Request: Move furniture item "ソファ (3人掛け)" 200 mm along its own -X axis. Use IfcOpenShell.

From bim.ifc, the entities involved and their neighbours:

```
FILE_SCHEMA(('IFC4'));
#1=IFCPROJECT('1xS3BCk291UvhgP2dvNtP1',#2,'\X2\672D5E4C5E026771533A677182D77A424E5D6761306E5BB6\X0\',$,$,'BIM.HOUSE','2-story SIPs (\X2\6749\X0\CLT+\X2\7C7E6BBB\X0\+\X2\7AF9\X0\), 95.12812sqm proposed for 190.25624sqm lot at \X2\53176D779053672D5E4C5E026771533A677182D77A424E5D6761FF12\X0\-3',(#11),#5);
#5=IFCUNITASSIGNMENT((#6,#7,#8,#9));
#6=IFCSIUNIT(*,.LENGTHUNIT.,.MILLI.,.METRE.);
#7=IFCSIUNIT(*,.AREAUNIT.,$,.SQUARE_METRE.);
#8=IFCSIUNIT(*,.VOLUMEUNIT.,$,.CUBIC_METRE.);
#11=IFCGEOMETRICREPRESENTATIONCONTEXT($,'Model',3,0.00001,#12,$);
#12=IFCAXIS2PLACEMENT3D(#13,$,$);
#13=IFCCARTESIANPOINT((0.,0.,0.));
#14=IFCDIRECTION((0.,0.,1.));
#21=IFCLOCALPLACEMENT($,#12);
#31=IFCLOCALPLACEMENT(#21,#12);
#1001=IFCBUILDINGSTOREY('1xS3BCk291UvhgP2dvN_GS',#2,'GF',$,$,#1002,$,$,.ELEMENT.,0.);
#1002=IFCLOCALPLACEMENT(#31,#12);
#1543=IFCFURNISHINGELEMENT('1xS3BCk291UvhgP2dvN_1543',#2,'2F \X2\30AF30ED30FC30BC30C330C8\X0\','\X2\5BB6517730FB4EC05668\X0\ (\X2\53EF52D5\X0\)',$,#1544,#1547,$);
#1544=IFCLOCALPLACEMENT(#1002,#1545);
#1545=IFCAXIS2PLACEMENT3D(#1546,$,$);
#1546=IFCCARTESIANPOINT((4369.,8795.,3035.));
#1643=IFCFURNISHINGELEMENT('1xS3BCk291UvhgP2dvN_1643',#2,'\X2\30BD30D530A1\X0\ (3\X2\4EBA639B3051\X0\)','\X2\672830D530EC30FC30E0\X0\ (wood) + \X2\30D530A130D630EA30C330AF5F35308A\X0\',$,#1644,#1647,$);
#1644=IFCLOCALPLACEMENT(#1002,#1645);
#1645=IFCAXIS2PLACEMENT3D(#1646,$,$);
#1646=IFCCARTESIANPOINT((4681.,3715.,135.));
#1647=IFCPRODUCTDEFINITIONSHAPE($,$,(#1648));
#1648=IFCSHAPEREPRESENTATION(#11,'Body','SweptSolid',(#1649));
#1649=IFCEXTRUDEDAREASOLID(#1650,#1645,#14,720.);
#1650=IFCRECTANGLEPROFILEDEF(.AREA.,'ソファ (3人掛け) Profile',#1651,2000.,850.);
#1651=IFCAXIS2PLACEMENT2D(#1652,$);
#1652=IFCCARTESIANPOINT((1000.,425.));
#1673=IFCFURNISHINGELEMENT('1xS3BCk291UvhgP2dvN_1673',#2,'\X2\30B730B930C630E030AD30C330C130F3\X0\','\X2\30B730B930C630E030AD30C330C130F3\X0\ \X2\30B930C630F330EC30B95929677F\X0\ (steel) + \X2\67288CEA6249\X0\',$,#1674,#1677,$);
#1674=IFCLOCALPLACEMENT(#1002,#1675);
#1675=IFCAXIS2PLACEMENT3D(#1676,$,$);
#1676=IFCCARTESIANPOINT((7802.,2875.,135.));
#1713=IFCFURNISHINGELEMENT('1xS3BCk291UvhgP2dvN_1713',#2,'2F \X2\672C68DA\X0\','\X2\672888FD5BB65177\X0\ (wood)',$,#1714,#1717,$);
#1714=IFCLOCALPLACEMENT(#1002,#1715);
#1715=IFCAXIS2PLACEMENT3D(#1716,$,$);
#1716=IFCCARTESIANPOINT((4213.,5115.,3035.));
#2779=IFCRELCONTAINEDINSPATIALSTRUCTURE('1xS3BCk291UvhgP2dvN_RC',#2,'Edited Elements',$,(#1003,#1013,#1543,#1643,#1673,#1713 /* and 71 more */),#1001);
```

```python
import ifcopenshell
import ifcopenshell.api.geometry
import ifcopenshell.util.placement
import ifcopenshell.util.unit

model = ifcopenshell.open("bim.ifc")
unit_scale = ifcopenshell.util.unit.calculate_unit_scale(model)

item = model.by_guid("1xS3BCk291UvhgP2dvN_1643")
matrix = ifcopenshell.util.placement.get_local_placement(item.ObjectPlacement)
matrix[:3, 3] -= matrix[:3, 0] * 0.2 / unit_scale
ifcopenshell.api.geometry.edit_object_placement(model, product=item, matrix=matrix, is_si=False)

print(ifcopenshell.util.placement.get_local_placement(item.ObjectPlacement).round(3) + 0.0)

model.write("bim_updated.ifc")
```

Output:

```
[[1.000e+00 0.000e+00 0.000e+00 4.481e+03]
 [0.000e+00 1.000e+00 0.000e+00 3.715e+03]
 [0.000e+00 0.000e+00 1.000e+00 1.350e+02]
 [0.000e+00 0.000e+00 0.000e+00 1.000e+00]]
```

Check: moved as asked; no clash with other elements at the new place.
